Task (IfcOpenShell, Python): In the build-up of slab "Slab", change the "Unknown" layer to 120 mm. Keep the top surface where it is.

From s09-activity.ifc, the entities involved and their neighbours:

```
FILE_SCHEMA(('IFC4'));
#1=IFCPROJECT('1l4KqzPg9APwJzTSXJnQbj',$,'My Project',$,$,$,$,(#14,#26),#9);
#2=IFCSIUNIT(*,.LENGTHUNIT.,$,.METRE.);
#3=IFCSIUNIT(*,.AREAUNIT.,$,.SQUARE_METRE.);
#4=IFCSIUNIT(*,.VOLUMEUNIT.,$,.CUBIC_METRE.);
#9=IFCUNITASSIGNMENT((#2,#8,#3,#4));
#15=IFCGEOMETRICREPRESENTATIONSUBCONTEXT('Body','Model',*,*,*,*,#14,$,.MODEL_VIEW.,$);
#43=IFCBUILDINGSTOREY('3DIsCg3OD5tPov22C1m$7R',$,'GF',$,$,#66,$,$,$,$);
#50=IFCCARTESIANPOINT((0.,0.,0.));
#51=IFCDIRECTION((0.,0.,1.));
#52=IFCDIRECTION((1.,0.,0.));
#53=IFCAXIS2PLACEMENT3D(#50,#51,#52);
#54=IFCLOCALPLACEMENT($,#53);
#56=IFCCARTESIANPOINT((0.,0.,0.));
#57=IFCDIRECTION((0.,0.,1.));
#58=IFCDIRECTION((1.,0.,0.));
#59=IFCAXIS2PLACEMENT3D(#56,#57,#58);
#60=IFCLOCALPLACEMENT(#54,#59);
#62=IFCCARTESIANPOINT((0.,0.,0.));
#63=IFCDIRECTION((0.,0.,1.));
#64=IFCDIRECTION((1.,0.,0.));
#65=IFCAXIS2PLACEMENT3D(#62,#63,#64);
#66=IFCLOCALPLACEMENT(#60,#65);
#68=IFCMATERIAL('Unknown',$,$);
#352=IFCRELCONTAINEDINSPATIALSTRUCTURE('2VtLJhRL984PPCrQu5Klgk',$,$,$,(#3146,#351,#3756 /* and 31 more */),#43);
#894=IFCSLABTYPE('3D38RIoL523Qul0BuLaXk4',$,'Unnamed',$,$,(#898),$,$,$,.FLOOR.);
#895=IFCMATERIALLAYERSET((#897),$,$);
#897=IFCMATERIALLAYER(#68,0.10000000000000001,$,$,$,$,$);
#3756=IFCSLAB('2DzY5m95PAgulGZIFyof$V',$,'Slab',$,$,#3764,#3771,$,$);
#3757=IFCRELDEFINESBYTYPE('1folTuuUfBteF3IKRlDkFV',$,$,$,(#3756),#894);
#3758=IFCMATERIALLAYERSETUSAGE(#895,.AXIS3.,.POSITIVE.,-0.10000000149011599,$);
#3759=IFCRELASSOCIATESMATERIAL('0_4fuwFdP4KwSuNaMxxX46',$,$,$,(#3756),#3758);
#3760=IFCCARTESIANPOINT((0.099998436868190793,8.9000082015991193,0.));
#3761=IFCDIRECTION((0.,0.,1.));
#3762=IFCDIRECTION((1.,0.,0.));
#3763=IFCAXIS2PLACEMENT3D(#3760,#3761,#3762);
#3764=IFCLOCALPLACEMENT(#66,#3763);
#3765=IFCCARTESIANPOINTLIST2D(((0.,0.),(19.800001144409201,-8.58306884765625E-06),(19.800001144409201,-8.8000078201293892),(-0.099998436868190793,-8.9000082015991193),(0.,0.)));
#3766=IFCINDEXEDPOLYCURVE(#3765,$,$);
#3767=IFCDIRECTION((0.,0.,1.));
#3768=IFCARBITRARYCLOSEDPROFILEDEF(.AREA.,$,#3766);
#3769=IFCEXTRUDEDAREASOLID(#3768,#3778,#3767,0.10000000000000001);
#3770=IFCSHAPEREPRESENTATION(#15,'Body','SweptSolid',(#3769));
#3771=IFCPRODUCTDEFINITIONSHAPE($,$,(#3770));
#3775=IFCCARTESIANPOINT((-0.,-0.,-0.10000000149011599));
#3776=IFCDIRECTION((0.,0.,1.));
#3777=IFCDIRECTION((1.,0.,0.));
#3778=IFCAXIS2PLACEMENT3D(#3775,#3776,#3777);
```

```python
import ifcopenshell
import ifcopenshell.util.element
import ifcopenshell.util.representation

model = ifcopenshell.open("s09-activity.ifc")

layer_set = model.by_id(895)
layer = next(l for l in layer_set.MaterialLayers if l.Material and l.Material.Name == "Unknown")
change = 0.12 - layer.LayerThickness
layer.LayerThickness += change

# Geometry does not follow the layer set by itself.
slabs = [e for e in ifcopenshell.util.element.get_elements_by_material(model, layer_set) if e.is_a("IfcSlab")]
for slab in sorted(slabs, key=lambda e: e.id()):
    body = ifcopenshell.util.representation.get_representation(slab, "Model", "Body")
    solid = body.Items[0]
    old_depth = solid.Depth
    solid.Depth += change
    # Extruded upwards: lower the start of the extrusion so the top stays.
    x, y, z = solid.Position.Location.Coordinates
    solid.Position.Location = model.createIfcCartesianPoint((x, y, z - change))
    print(slab.id(), f"{old_depth:g} -> {solid.Depth:g}")

# The layers are counted up from the underside, which has moved.
for usage in {ifcopenshell.util.element.get_material(slab) for slab in slabs}:
    usage.OffsetFromReferenceLine -= change

model.write("s09-activity-out.ifc")
```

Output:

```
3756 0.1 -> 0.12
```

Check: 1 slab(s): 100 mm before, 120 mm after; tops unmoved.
